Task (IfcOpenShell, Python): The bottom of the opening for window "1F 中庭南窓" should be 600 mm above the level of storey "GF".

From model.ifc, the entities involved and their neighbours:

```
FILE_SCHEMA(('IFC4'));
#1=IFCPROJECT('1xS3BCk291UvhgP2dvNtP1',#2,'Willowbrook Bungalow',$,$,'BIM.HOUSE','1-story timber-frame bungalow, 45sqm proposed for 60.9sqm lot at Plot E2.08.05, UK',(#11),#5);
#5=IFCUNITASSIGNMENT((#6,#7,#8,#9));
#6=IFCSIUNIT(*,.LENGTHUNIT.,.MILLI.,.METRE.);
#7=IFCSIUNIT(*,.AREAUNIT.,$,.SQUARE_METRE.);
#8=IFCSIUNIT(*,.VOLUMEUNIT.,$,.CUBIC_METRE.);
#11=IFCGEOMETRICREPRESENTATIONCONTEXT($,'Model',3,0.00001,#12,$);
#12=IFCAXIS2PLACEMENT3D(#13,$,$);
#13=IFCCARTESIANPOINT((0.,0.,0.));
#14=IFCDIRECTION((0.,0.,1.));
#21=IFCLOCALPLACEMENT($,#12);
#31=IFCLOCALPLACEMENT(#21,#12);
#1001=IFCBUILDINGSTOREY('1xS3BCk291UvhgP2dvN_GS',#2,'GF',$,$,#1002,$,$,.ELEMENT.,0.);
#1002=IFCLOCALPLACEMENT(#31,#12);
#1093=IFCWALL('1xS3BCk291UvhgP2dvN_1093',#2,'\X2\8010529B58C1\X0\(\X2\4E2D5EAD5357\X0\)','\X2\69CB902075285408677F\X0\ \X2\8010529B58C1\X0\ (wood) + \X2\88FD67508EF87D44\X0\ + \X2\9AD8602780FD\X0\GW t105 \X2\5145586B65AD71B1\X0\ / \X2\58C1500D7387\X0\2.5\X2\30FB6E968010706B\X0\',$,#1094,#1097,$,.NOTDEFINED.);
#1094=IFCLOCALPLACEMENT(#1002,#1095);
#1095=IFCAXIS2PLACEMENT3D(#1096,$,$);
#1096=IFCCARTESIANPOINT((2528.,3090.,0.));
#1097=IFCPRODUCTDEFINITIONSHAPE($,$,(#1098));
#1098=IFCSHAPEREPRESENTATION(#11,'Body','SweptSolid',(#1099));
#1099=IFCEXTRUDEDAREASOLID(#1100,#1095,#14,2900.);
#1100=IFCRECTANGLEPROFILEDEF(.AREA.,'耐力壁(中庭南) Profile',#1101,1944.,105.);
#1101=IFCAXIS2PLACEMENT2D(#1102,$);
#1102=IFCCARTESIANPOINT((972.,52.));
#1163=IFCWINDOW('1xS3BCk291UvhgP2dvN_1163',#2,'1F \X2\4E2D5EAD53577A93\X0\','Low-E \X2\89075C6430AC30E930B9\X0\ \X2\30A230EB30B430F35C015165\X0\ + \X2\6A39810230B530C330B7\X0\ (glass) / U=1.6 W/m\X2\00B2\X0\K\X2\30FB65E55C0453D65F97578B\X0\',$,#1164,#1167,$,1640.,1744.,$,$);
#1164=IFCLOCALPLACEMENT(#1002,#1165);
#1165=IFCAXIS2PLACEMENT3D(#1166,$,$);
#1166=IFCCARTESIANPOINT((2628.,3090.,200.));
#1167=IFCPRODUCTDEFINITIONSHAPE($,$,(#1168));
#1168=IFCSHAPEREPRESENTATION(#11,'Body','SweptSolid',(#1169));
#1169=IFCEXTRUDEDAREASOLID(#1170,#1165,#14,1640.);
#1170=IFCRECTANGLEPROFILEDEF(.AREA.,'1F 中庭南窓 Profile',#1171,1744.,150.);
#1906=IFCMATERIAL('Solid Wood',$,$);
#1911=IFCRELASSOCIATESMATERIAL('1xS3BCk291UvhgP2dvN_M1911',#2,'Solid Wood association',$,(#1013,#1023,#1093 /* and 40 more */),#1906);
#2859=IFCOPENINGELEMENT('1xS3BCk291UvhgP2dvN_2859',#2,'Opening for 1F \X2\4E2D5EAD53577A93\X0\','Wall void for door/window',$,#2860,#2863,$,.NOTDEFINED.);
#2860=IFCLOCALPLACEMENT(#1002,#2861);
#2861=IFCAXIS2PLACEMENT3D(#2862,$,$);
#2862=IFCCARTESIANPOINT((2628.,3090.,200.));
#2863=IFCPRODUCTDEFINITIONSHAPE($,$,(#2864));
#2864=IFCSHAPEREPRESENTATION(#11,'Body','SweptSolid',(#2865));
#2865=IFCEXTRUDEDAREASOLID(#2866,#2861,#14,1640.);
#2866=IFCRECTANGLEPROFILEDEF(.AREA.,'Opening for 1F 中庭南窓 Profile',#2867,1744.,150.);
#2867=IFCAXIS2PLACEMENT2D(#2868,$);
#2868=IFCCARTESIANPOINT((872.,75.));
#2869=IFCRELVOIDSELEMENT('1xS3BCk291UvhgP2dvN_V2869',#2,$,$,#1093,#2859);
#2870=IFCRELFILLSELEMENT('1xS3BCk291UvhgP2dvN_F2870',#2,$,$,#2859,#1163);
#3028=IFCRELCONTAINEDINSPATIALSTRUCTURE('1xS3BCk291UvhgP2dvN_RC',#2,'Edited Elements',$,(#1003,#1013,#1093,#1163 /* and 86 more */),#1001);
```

```python
import numpy as np
import ifcopenshell
import ifcopenshell.api.geometry
import ifcopenshell.geom
import ifcopenshell.util.element
import ifcopenshell.util.placement
import ifcopenshell.util.shape
import ifcopenshell.util.unit

model = ifcopenshell.open("model.ifc")
unit_scale = ifcopenshell.util.unit.calculate_unit_scale(model)

window = model.by_guid("1xS3BCk291UvhgP2dvN_1163")
opening = window.FillsVoids[0].RelatingOpeningElement
storey = ifcopenshell.util.element.get_container(window, ifc_class="IfcBuildingStorey")
level = ifcopenshell.util.placement.get_local_placement(storey.ObjectPlacement)[2, 3]

# The opening's origin need not be at the sill, so measure its lowest point.
shape = ifcopenshell.geom.create_shape(ifcopenshell.geom.settings(), opening)
bottom = ifcopenshell.util.shape.get_shape_bottom_elevation(shape, shape.geometry) / unit_scale
dz = level + 0.6 / unit_scale - bottom

shift = np.array([0.0, 0.0, dz])
# The window is not placed relative to its opening, so move both.
for product in (opening, window):
    matrix = ifcopenshell.util.placement.get_local_placement(product.ObjectPlacement)
    matrix[:3, 3] += shift
    ifcopenshell.api.geometry.edit_object_placement(model, product=product, matrix=matrix, is_si=False)

print(f"moved by {dz * unit_scale:+.3f} m")

model.write("model_v2.ifc")
```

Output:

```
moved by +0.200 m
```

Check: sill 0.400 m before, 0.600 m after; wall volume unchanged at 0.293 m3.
